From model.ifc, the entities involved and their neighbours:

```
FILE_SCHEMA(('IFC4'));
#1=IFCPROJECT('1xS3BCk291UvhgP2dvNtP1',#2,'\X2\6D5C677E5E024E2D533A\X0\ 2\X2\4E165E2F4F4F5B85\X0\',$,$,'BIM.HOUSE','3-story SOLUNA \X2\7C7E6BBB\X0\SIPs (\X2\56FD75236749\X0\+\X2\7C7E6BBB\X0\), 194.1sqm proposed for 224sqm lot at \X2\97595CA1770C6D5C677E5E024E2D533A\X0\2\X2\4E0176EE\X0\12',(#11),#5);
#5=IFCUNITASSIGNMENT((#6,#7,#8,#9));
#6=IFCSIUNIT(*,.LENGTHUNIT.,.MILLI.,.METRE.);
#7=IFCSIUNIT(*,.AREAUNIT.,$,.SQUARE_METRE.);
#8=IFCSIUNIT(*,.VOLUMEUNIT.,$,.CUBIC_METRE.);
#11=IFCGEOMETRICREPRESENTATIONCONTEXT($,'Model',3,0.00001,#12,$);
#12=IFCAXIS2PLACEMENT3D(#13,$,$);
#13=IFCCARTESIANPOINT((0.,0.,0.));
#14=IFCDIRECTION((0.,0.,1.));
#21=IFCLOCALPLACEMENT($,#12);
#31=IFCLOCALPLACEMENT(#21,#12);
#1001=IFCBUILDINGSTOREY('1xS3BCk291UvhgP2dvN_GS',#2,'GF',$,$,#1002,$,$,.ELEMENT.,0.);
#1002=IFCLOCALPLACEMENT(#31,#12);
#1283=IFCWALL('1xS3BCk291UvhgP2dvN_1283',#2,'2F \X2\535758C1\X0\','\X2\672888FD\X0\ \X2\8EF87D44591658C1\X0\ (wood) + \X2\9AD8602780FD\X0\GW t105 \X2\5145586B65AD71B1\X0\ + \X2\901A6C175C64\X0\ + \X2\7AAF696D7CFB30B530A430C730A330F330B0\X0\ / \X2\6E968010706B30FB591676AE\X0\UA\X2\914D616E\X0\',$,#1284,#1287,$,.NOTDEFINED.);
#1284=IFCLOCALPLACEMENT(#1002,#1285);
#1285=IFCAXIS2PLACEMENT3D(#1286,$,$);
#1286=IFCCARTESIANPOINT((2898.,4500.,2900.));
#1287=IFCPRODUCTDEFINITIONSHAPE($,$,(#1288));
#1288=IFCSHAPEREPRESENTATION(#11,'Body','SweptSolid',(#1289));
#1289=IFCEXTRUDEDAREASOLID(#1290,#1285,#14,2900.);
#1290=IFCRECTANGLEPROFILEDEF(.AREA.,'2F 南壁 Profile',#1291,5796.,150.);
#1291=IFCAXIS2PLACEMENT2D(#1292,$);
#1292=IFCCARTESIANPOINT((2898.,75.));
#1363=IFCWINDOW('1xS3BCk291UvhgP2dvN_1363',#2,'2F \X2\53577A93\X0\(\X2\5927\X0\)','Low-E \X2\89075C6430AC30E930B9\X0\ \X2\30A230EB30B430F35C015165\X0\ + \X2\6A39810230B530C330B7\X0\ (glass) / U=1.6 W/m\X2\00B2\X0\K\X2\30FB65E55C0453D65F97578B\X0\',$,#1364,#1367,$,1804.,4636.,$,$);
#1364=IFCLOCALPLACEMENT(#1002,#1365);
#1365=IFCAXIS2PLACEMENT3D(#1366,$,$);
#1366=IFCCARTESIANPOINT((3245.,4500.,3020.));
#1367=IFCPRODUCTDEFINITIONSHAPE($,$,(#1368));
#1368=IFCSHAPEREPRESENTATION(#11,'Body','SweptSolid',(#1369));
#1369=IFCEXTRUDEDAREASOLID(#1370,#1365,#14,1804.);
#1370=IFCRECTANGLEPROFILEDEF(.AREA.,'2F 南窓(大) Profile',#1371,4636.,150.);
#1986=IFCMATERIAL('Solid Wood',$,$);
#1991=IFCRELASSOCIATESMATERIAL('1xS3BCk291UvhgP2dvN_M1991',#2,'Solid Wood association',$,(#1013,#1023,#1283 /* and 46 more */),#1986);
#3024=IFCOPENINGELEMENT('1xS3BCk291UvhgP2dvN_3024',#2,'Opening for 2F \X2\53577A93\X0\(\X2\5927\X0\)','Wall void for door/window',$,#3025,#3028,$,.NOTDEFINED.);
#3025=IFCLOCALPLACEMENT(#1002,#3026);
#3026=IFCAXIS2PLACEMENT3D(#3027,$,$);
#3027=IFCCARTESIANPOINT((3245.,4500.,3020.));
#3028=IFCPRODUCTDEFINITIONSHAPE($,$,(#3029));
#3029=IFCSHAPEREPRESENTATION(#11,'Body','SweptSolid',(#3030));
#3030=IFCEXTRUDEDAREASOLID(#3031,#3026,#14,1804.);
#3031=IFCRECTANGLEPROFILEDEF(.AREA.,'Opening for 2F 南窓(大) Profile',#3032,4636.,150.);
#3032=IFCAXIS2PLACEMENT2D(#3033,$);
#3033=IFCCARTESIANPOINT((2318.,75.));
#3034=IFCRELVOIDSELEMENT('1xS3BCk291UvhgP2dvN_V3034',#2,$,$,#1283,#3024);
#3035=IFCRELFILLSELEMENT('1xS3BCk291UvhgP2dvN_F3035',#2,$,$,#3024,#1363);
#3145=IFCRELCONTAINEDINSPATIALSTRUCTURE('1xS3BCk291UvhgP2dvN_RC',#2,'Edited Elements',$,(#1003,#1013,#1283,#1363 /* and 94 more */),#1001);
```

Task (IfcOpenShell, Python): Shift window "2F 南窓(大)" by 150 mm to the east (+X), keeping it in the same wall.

```python
import ifcopenshell
import ifcopenshell.api.geometry
import ifcopenshell.util.placement

model = ifcopenshell.open("model.ifc")

window = model.by_guid("1xS3BCk291UvhgP2dvN_1363")
opening = window.FillsVoids[0].RelatingOpeningElement
wall = opening.VoidsElements[0].RelatingBuildingElement

wall_matrix = ifcopenshell.util.placement.get_local_placement(wall.ObjectPlacement)
shift = wall_matrix[:3, 0] * 150.0
before = ifcopenshell.util.placement.get_local_placement(window.ObjectPlacement)[:3, 3].copy()

# The window is not placed relative to its opening, so move both.
for product in (opening, window):
    matrix = ifcopenshell.util.placement.get_local_placement(product.ObjectPlacement)
    matrix[:3, 3] += shift
    ifcopenshell.api.geometry.edit_object_placement(model, product=product, matrix=matrix, is_si=False)

after = ifcopenshell.util.placement.get_local_placement(window.ObjectPlacement)[:3, 3]
print("window moved by", (after - before).round(3) + 0.0)

model.write("model-out.ifc")
```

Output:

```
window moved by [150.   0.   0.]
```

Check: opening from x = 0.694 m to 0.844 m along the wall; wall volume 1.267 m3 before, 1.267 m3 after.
